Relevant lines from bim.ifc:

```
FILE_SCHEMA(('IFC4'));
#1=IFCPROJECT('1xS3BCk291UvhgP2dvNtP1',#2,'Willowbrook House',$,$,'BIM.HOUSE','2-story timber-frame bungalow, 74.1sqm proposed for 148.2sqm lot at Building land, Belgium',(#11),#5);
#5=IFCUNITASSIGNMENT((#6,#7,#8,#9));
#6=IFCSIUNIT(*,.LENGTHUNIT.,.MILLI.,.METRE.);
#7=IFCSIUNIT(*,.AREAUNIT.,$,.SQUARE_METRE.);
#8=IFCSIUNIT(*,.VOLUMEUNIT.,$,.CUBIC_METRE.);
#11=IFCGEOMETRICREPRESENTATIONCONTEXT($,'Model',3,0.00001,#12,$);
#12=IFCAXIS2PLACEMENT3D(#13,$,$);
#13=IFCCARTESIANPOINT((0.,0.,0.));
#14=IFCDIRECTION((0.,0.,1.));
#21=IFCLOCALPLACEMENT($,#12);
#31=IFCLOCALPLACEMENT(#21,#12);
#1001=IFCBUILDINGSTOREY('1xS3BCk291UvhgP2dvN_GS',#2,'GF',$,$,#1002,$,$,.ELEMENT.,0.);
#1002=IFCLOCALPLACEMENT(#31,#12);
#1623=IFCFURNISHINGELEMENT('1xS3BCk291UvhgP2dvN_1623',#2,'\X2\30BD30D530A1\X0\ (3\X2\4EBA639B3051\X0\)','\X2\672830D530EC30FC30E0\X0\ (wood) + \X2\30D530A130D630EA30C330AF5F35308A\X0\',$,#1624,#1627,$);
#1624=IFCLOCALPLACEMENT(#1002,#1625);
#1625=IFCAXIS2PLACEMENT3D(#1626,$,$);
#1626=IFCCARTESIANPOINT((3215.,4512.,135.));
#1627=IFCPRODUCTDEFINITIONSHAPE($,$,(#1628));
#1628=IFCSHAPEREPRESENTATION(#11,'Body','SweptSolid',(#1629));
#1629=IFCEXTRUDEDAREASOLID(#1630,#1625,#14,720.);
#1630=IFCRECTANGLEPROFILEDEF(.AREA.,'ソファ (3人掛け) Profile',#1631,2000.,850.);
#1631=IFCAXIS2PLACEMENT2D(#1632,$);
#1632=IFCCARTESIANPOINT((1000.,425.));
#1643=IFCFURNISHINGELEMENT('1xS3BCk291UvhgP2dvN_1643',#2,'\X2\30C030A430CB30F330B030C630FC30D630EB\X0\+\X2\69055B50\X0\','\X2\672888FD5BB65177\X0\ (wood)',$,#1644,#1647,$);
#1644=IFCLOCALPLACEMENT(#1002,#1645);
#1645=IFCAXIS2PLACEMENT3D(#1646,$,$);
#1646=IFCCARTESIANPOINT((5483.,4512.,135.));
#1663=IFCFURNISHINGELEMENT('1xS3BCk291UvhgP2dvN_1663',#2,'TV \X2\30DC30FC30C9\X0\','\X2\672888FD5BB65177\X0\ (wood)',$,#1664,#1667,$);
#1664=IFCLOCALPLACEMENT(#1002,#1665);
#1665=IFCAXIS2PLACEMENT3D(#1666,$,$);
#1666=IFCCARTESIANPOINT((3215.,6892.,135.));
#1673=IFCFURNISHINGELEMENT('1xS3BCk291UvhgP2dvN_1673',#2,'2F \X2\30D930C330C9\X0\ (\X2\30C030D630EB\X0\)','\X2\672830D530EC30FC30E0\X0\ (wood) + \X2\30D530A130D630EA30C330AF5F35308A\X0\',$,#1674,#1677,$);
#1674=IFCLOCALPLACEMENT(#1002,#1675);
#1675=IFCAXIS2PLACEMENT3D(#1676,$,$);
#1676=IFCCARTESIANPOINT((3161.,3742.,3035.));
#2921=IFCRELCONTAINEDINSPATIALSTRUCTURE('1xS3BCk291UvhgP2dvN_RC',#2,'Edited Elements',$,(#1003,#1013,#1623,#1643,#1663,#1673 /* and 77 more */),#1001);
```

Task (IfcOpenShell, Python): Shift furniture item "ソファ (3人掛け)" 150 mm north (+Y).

```python
import ifcopenshell
import ifcopenshell.api.geometry
import ifcopenshell.util.placement

model = ifcopenshell.open("bim.ifc")

item = model.by_id(1623)
matrix = ifcopenshell.util.placement.get_local_placement(item.ObjectPlacement)
matrix[1, 3] += 150.0
ifcopenshell.api.geometry.edit_object_placement(model, product=item, matrix=matrix, is_si=False)

print(ifcopenshell.util.placement.get_local_placement(item.ObjectPlacement).round(3) + 0.0)

model.write("bim-out.ifc")
```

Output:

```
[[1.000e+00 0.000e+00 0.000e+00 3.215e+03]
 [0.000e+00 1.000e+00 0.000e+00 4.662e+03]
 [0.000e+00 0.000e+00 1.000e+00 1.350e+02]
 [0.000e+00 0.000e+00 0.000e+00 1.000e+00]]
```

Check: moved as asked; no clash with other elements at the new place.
